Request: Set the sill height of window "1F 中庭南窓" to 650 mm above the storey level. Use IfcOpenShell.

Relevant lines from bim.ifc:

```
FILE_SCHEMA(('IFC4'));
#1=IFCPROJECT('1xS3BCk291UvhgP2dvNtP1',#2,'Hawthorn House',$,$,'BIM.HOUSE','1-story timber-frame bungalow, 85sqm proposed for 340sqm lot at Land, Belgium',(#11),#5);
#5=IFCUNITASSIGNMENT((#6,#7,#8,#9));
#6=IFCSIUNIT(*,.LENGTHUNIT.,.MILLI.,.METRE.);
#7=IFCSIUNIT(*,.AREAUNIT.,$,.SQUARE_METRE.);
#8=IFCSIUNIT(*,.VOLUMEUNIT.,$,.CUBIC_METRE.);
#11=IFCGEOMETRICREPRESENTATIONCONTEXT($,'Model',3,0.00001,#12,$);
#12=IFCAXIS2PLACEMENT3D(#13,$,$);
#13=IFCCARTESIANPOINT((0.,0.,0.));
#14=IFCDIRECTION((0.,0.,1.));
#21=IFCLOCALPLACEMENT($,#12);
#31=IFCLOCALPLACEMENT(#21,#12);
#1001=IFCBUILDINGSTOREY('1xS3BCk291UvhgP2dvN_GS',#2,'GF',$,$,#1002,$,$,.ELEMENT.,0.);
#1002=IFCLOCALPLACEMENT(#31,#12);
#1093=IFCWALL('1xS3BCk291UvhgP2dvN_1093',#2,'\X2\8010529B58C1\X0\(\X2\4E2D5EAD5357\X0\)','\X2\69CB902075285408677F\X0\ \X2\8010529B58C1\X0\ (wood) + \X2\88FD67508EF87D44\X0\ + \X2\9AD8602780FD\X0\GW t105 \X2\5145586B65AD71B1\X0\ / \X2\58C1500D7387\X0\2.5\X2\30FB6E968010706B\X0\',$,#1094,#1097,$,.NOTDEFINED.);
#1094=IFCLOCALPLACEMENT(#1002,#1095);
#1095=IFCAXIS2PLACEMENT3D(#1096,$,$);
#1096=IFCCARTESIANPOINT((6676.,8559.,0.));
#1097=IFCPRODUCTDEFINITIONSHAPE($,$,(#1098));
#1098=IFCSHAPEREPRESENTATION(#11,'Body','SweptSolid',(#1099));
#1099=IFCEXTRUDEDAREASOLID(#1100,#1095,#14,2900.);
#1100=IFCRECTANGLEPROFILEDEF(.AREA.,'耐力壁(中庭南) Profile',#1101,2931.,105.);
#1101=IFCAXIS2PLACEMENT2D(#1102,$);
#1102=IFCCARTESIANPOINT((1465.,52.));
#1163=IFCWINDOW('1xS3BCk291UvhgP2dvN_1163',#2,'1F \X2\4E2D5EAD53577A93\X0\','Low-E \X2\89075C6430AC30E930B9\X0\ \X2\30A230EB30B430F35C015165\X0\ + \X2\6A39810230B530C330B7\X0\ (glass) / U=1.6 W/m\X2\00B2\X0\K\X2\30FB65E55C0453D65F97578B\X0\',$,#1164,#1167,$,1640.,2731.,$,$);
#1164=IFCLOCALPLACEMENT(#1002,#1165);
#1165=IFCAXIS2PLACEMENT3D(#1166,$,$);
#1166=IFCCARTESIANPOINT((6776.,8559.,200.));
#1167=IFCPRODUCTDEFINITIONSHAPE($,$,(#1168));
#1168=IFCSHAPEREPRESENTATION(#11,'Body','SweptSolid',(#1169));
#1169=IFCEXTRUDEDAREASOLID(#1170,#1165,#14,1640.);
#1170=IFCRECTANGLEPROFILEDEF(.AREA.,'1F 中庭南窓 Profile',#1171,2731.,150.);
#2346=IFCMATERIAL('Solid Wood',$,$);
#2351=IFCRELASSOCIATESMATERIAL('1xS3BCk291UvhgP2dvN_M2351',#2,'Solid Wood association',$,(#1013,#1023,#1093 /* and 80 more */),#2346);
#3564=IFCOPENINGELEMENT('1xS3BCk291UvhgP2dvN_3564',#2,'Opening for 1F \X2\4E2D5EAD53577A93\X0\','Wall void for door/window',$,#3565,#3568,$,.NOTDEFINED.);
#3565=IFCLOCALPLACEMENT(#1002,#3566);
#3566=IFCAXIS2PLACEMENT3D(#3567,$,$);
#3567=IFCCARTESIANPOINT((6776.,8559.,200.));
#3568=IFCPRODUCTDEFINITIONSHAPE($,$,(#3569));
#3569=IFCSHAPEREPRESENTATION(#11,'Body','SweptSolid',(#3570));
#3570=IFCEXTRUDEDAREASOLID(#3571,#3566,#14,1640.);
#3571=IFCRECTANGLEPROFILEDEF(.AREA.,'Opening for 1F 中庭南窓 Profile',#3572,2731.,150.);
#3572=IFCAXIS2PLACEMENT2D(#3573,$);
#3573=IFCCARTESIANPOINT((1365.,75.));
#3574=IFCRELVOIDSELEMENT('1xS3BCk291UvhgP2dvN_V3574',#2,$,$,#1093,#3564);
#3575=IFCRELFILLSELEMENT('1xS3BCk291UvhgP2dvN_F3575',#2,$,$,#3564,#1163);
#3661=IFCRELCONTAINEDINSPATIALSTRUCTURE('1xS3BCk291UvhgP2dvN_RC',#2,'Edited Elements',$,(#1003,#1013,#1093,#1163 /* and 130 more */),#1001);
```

```python
import numpy as np
import ifcopenshell
import ifcopenshell.api.geometry
import ifcopenshell.geom
import ifcopenshell.util.element
import ifcopenshell.util.placement
import ifcopenshell.util.shape
import ifcopenshell.util.unit

model = ifcopenshell.open("bim.ifc")
unit_scale = ifcopenshell.util.unit.calculate_unit_scale(model)

window = model.by_id(1163)
opening = window.FillsVoids[0].RelatingOpeningElement
storey = ifcopenshell.util.element.get_container(window, ifc_class="IfcBuildingStorey")
level = ifcopenshell.util.placement.get_local_placement(storey.ObjectPlacement)[2, 3]

# The opening's origin need not be at the sill, so measure its lowest point.
shape = ifcopenshell.geom.create_shape(ifcopenshell.geom.settings(), opening)
bottom = ifcopenshell.util.shape.get_shape_bottom_elevation(shape, shape.geometry) / unit_scale
dz = level + 0.65 / unit_scale - bottom

shift = np.array([0.0, 0.0, dz])
# The window is not placed relative to its opening, so move both.
for product in (opening, window):
    matrix = ifcopenshell.util.placement.get_local_placement(product.ObjectPlacement)
    matrix[:3, 3] += shift
    ifcopenshell.api.geometry.edit_object_placement(model, product=product, matrix=matrix, is_si=False)

print(f"moved by {dz * unit_scale:+.3f} m")

model.write("bim_v2.ifc")
```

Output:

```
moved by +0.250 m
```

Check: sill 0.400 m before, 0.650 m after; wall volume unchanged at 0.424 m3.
